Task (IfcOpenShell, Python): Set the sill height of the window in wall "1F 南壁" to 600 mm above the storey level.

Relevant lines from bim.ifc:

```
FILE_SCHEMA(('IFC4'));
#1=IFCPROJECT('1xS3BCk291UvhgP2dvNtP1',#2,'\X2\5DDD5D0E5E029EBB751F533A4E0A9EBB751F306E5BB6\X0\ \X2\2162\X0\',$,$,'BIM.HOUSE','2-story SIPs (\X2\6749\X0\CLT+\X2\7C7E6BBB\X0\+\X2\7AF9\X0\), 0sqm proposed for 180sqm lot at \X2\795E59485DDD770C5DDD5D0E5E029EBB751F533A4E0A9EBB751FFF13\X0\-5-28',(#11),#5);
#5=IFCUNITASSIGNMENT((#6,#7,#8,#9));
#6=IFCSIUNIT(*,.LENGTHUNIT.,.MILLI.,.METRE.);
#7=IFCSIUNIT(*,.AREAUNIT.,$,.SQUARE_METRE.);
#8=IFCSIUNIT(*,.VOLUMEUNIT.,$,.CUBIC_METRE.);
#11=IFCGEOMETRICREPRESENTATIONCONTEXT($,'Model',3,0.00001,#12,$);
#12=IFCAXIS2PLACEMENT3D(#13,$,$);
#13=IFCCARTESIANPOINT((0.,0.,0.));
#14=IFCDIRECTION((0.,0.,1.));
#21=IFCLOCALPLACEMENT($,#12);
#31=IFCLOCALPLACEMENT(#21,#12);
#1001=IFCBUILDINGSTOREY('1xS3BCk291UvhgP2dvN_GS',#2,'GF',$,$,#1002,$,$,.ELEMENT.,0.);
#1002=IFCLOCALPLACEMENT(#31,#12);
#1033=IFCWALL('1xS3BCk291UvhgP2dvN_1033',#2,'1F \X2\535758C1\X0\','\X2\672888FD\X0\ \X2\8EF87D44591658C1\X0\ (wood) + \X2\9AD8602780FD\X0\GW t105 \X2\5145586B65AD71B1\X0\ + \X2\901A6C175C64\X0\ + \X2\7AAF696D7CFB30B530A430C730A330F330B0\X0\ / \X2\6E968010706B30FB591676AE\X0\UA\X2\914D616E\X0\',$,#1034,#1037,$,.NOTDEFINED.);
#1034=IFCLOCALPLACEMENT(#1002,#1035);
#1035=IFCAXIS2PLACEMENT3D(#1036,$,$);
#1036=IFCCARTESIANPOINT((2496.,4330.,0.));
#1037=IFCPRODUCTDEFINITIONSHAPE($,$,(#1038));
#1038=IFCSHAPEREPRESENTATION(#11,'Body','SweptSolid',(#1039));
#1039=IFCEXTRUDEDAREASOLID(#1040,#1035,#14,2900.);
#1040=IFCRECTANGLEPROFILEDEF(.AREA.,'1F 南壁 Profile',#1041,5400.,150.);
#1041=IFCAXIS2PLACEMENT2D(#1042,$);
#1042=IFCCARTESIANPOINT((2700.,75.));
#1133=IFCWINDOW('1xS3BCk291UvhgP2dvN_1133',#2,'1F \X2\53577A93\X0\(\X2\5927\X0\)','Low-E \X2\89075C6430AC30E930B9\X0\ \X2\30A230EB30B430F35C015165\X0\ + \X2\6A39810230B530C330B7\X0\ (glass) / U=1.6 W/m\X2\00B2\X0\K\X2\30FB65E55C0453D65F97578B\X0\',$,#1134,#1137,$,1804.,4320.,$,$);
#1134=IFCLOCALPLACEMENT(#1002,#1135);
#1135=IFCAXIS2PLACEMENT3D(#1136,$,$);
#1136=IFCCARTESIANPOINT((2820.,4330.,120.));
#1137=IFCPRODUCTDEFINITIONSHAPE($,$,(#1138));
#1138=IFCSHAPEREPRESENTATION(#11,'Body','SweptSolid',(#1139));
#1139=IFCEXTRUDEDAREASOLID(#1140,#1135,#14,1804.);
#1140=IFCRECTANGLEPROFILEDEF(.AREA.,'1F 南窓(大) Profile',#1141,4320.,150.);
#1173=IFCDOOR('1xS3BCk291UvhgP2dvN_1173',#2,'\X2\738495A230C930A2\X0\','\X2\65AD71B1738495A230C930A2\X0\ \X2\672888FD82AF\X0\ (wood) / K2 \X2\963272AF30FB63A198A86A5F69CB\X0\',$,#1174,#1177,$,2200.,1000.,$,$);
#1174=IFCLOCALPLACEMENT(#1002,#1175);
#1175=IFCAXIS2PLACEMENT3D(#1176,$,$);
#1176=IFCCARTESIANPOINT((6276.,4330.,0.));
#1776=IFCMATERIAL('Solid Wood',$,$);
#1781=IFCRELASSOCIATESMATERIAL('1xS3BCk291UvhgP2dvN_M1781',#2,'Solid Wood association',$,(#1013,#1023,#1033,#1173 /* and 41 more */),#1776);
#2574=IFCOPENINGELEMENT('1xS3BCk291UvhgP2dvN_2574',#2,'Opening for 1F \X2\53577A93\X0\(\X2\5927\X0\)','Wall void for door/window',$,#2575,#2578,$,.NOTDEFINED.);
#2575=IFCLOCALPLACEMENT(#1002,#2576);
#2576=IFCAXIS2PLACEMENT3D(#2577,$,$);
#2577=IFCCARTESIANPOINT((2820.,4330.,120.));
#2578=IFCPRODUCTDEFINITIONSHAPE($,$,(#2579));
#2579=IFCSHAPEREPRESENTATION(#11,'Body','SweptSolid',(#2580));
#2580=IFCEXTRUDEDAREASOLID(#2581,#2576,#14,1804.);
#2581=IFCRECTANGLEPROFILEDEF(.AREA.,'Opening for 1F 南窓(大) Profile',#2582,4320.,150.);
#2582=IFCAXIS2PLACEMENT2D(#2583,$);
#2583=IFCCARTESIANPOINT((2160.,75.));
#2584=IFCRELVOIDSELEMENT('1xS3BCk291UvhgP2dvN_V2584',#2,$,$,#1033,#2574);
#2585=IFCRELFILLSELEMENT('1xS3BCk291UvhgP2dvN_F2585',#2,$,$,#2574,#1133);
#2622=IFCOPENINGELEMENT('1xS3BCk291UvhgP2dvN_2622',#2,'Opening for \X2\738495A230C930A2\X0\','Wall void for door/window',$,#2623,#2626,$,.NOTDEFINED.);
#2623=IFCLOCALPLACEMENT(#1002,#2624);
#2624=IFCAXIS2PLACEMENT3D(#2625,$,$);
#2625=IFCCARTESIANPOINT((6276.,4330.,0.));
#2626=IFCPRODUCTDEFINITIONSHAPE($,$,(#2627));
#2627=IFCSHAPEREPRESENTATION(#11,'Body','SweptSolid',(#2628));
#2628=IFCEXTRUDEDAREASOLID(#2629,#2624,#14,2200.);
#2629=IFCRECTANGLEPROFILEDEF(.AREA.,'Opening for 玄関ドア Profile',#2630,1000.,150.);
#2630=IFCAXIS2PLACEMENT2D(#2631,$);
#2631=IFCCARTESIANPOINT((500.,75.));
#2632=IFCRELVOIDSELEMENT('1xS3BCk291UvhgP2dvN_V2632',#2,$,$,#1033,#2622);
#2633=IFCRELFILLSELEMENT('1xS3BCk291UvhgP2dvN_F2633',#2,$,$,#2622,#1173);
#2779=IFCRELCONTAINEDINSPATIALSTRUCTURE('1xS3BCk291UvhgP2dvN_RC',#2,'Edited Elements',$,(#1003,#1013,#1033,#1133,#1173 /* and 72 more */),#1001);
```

```python
import numpy as np
import ifcopenshell
import ifcopenshell.api.geometry
import ifcopenshell.geom
import ifcopenshell.util.element
import ifcopenshell.util.placement
import ifcopenshell.util.shape
import ifcopenshell.util.unit

model = ifcopenshell.open("bim.ifc")
unit_scale = ifcopenshell.util.unit.calculate_unit_scale(model)

window = model.by_id(1133)
opening = window.FillsVoids[0].RelatingOpeningElement
storey = ifcopenshell.util.element.get_container(window, ifc_class="IfcBuildingStorey")
level = ifcopenshell.util.placement.get_local_placement(storey.ObjectPlacement)[2, 3]

# The opening's origin need not be at the sill, so measure its lowest point.
shape = ifcopenshell.geom.create_shape(ifcopenshell.geom.settings(), opening)
bottom = ifcopenshell.util.shape.get_shape_bottom_elevation(shape, shape.geometry) / unit_scale
dz = level + 0.6 / unit_scale - bottom

shift = np.array([0.0, 0.0, dz])
# The window is not placed relative to its opening, so move both.
for product in (opening, window):
    matrix = ifcopenshell.util.placement.get_local_placement(product.ObjectPlacement)
    matrix[:3, 3] += shift
    ifcopenshell.api.geometry.edit_object_placement(model, product=product, matrix=matrix, is_si=False)

print(f"moved by {dz * unit_scale:+.3f} m")

model.write("bim_edited.ifc")
```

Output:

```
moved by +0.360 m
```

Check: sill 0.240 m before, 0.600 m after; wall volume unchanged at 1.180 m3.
